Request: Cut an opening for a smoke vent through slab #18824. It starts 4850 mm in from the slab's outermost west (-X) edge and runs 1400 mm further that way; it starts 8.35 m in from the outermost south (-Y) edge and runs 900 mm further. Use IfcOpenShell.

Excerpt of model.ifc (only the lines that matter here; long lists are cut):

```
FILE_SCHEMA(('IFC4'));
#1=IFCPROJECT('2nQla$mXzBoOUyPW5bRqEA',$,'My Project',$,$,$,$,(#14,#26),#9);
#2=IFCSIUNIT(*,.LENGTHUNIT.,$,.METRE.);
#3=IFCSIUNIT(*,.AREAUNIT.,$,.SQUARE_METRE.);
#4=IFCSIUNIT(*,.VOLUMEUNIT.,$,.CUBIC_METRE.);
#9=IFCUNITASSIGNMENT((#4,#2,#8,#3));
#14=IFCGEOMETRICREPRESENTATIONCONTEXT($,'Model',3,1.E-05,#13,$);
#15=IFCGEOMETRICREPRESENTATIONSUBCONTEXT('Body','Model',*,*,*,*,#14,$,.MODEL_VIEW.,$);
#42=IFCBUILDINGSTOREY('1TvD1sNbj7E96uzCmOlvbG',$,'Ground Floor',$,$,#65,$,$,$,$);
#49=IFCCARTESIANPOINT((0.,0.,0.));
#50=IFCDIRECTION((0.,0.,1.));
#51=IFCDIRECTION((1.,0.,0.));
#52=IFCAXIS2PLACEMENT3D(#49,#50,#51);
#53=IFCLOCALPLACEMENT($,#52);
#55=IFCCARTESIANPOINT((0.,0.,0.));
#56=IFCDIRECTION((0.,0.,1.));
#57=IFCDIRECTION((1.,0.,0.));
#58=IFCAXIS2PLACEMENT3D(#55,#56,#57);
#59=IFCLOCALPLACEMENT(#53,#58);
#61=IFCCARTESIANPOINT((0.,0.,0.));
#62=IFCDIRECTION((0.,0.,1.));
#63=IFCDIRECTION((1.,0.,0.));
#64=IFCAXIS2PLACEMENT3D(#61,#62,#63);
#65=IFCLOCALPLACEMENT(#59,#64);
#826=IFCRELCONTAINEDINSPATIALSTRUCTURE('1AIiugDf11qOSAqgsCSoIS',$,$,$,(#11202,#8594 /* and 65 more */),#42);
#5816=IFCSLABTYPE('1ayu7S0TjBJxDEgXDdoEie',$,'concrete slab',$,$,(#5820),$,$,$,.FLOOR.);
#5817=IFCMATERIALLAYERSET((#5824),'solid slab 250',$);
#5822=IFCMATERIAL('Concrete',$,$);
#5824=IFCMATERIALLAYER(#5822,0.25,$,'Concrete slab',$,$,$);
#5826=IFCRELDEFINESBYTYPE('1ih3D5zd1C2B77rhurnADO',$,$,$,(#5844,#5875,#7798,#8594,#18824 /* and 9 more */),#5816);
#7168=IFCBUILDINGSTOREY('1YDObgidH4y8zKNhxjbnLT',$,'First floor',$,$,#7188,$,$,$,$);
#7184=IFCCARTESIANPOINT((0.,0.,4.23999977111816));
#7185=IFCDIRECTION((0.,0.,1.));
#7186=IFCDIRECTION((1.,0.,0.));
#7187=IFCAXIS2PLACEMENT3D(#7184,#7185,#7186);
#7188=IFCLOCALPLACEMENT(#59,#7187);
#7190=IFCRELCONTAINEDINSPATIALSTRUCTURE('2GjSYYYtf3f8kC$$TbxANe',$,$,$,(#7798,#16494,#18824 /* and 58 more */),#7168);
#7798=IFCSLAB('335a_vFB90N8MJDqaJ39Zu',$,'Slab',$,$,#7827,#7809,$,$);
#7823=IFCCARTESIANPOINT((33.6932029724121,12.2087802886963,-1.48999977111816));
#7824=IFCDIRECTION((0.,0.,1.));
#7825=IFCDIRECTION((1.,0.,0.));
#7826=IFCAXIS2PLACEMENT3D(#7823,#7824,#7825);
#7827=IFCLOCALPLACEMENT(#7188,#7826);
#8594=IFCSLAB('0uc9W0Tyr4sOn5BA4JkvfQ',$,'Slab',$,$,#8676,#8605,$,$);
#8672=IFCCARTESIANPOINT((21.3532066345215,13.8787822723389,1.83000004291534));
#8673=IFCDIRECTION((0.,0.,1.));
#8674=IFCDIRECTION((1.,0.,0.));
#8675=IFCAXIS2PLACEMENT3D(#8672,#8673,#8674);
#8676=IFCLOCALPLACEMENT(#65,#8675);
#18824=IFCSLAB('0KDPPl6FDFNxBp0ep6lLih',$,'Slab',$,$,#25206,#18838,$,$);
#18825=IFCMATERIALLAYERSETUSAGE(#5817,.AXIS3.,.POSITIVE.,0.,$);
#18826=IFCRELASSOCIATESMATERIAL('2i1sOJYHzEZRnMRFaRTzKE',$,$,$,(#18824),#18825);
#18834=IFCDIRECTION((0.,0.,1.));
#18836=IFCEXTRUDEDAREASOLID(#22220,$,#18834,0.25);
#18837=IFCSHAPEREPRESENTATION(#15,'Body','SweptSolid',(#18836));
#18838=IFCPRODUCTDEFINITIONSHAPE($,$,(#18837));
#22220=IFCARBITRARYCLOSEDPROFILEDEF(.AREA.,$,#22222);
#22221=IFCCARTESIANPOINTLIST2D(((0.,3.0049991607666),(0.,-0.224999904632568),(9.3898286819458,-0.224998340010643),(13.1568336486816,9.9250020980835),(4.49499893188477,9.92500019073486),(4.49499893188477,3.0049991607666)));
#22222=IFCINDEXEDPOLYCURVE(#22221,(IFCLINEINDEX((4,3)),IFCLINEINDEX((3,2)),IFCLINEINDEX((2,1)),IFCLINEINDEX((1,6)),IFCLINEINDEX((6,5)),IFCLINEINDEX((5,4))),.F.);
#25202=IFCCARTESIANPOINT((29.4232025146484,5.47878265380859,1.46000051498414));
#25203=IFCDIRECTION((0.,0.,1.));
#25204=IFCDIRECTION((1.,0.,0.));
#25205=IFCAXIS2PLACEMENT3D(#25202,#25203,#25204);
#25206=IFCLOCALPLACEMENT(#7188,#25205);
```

```python
import numpy as np
import ifcopenshell
import ifcopenshell.api.feature
import ifcopenshell.api.geometry
import ifcopenshell.api.root
import ifcopenshell.geom
import ifcopenshell.util.placement
import ifcopenshell.util.representation
import ifcopenshell.util.shape
import ifcopenshell.util.unit

model = ifcopenshell.open("model.ifc")
unit_scale = ifcopenshell.util.unit.calculate_unit_scale(model)
settings = ifcopenshell.geom.settings()


def volume(element):
    """Net volume in cubic metres, openings subtracted."""
    shape = ifcopenshell.geom.create_shape(settings, element)
    return ifcopenshell.util.shape.get_volume(shape.geometry)


slab = model.by_guid("0KDPPl6FDFNxBp0ep6lLih")
before = volume(slab)

# Extent in the slab's own axes, in metres. The edges named are its -X and -Y sides.
slab_shape = ifcopenshell.geom.create_shape(settings, slab)
vertices = ifcopenshell.util.shape.get_vertices(slab_shape.geometry)
x_min, y_min, bottom = vertices.min(axis=0)
top = vertices[:, 2].max()

opening = ifcopenshell.api.root.create_entity(model, ifc_class="IfcOpeningElement", name="Smoke vent opening", predefined_type="OPENING")
context = ifcopenshell.util.representation.get_context(model, "Model", "Body", "MODEL_VIEW")
width, depth = 1.4, 0.9
outline = [(0.0, 0.0), (width, 0.0), (width, depth), (0.0, depth), (0.0, 0.0)]
# Overshoot both faces by 50 mm so the cut is clean.
shape = ifcopenshell.api.geometry.add_slab_representation(
    model, context=context, depth=top - bottom + 0.1, polyline=outline
)
ifcopenshell.api.geometry.assign_representation(model, product=opening, representation=shape)

matrix = ifcopenshell.util.placement.get_local_placement(slab.ObjectPlacement)
matrix[:, 3] = matrix @ np.append(np.array([x_min + 4.85, y_min + 8.35, bottom - 0.05]) / unit_scale, 1.0)
ifcopenshell.api.geometry.edit_object_placement(model, product=opening, matrix=matrix, is_si=False)
ifcopenshell.api.feature.add_feature(model, feature=opening, element=slab)

after = volume(slab)

print(f"slab volume {before:.3f} -> {after:.3f} m3")

model.write("model_updated.ifc")
```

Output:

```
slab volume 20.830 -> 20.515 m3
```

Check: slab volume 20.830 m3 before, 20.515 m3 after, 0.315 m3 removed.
